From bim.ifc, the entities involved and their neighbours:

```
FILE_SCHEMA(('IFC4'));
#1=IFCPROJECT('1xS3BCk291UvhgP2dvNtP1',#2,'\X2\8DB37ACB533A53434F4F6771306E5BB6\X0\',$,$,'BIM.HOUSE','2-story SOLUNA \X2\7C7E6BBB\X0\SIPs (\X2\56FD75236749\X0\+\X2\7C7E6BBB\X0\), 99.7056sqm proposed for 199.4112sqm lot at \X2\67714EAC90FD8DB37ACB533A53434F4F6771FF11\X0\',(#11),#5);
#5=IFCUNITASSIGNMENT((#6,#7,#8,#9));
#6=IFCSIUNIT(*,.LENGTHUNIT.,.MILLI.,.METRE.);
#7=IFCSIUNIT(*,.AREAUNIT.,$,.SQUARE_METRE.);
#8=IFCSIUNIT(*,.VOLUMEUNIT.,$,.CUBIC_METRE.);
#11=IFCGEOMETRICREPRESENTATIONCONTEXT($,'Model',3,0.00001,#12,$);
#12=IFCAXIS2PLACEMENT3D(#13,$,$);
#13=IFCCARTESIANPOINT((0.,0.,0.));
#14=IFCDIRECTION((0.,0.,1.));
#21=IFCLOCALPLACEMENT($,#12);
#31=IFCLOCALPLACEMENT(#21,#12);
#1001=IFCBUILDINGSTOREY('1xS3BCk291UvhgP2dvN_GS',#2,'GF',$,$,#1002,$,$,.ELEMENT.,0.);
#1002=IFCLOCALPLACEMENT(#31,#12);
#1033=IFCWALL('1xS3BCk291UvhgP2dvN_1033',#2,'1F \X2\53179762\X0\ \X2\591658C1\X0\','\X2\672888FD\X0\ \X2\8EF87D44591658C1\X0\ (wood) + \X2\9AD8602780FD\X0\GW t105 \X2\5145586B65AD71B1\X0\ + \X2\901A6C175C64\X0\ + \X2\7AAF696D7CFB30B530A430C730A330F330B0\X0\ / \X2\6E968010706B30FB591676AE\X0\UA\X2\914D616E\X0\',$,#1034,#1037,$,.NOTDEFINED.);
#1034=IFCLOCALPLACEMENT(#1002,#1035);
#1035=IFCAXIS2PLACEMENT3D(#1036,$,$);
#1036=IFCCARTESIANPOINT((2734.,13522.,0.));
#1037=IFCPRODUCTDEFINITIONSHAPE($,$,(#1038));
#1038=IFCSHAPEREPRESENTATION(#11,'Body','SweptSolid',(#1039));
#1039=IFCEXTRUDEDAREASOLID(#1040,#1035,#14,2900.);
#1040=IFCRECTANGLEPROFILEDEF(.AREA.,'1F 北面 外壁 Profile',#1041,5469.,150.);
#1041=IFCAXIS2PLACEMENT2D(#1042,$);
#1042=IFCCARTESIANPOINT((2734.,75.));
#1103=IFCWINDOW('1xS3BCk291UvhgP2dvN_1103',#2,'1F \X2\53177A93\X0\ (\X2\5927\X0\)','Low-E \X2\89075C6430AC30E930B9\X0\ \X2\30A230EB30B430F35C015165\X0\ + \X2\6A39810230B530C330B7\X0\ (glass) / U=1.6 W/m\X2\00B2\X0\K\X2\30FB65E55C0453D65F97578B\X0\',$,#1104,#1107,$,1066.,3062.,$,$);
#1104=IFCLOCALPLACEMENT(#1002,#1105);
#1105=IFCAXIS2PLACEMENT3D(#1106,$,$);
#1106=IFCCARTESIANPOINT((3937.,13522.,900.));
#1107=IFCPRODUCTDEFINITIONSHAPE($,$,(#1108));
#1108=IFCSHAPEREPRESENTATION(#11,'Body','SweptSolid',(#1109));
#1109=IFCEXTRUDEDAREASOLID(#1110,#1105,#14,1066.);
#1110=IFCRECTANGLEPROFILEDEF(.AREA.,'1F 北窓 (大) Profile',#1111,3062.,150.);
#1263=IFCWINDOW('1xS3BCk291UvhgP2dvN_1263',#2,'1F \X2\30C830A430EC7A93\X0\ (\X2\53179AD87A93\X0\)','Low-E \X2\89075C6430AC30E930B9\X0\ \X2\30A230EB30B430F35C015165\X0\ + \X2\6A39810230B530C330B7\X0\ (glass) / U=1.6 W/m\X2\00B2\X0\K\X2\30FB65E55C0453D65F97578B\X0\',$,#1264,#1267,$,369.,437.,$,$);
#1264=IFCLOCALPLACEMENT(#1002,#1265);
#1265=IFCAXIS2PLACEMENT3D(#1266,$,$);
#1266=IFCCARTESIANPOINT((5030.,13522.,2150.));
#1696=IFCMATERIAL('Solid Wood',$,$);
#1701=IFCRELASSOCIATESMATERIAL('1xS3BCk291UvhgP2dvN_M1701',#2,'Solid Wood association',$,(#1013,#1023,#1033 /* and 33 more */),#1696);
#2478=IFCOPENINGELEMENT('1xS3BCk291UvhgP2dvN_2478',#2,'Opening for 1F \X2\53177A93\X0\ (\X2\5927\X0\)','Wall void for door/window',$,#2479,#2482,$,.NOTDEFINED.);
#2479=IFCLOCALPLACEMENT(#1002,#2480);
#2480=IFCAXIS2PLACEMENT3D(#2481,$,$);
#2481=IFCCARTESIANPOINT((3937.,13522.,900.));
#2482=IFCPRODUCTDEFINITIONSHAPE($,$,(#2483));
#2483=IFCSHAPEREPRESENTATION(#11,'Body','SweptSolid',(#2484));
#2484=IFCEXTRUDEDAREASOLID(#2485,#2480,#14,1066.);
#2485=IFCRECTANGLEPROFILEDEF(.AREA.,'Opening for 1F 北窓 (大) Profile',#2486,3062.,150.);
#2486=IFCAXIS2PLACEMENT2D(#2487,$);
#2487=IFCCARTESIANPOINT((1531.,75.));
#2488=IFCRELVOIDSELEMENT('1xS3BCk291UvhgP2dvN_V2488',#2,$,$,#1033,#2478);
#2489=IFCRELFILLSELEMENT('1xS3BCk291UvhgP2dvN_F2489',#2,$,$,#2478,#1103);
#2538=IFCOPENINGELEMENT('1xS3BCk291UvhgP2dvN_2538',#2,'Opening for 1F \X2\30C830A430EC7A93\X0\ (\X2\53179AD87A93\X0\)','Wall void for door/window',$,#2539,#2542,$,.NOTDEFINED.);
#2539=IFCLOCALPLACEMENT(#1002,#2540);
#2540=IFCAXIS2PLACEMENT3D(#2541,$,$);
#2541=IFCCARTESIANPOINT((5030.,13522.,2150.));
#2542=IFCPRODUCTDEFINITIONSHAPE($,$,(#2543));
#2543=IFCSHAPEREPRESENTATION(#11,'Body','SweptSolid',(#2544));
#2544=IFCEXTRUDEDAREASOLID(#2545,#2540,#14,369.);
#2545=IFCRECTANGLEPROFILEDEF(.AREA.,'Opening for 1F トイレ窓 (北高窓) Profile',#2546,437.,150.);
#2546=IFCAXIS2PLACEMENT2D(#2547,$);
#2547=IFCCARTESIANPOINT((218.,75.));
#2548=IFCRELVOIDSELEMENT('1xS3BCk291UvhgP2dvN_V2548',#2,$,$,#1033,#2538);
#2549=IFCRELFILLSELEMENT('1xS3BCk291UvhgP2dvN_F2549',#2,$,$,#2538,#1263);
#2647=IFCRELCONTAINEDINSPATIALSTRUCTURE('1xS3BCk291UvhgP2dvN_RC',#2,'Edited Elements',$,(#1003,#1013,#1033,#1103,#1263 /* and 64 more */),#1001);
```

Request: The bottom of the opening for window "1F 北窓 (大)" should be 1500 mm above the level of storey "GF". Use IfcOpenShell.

```python
import numpy as np
import ifcopenshell
import ifcopenshell.api.geometry
import ifcopenshell.geom
import ifcopenshell.util.element
import ifcopenshell.util.placement
import ifcopenshell.util.shape
import ifcopenshell.util.unit

model = ifcopenshell.open("bim.ifc")
unit_scale = ifcopenshell.util.unit.calculate_unit_scale(model)

window = model.by_id(1103)
opening = window.FillsVoids[0].RelatingOpeningElement
storey = ifcopenshell.util.element.get_container(window, ifc_class="IfcBuildingStorey")
level = ifcopenshell.util.placement.get_local_placement(storey.ObjectPlacement)[2, 3]

# The opening's origin need not be at the sill, so measure its lowest point.
shape = ifcopenshell.geom.create_shape(ifcopenshell.geom.settings(), opening)
bottom = ifcopenshell.util.shape.get_shape_bottom_elevation(shape, shape.geometry) / unit_scale
dz = level + 1.5 / unit_scale - bottom

shift = np.array([0.0, 0.0, dz])
# The window is not placed relative to its opening, so move both.
for product in (opening, window):
    matrix = ifcopenshell.util.placement.get_local_placement(product.ObjectPlacement)
    matrix[:3, 3] += shift
    ifcopenshell.api.geometry.edit_object_placement(model, product=product, matrix=matrix, is_si=False)

print(f"moved by {dz * unit_scale:+.3f} m")

model.write("bim_v2.ifc")
```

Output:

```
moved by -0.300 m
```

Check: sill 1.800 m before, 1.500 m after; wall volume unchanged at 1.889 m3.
